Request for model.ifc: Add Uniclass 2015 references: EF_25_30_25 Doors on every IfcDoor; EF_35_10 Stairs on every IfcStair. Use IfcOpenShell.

First a look at what the model holds.

```python
import ifcopenshell

model = ifcopenshell.open("model.ifc")
print(model.schema)
print("classifications:", [c.Name for c in model.by_type("IfcClassification")])
for ifc_class in ("IfcDoor", "IfcRoof", "IfcStair", "IfcWall", "IfcWindow"):
    print(ifc_class, len(model.by_type(ifc_class)))
```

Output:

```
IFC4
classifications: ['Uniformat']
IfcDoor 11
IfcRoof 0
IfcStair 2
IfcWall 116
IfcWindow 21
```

```python
import ifcopenshell
import ifcopenshell.api.classification

model = ifcopenshell.open("model.ifc")

system = ifcopenshell.api.classification.add_classification(model, classification="Uniclass 2015")

codes = {
    "IfcDoor": ("EF_25_30_25", "Doors"),
    "IfcStair": ("EF_35_10", "Stairs"),
}
for ifc_class, (code, name) in codes.items():
    products = model.by_type(ifc_class)
    ifcopenshell.api.classification.add_reference(
        model, products=products, classification=system, identification=code, name=name
    )
    print(code, len(products))

model.write("model_v2.ifc")
```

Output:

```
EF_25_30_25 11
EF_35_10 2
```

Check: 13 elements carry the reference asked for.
